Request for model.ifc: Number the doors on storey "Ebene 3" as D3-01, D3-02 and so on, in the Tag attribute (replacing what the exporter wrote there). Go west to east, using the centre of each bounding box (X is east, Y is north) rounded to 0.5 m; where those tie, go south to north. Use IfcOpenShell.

First a look at what the model holds.

```python
import ifcopenshell
import ifcopenshell.util.element
import ifcopenshell.util.placement

model = ifcopenshell.open("model.ifc")
print(model.schema)
storey = next(s for s in model.by_type("IfcBuildingStorey") if s.Name == "Ebene 3")
doors = [e for e in ifcopenshell.util.element.get_decomposition(storey) if e.is_a("IfcDoor")]
for e in sorted(doors, key=lambda e: e.id()):
    origin = ifcopenshell.util.placement.get_local_placement(e.ObjectPlacement)[:3, 3]
    print(e.id(), e.Tag, e.Name, origin.round(2) + 0.0, sep=" | ")
```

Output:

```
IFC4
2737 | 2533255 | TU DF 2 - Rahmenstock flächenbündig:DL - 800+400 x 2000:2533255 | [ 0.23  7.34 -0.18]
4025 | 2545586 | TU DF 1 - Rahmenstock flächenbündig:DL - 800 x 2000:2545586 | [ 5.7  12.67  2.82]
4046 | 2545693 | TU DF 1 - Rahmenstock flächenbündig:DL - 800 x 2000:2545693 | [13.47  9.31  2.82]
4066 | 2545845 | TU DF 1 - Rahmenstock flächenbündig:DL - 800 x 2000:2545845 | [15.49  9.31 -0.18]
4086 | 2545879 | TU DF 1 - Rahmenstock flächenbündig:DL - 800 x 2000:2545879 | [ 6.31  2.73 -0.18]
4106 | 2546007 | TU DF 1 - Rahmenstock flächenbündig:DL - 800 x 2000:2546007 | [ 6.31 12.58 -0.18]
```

```python
import ifcopenshell
import ifcopenshell.geom
import ifcopenshell.util.element
import ifcopenshell.util.shape

model = ifcopenshell.open("model.ifc")
settings = ifcopenshell.geom.settings()
settings.set("use-world-coords", True)


def centre(element):
    shape = ifcopenshell.geom.create_shape(settings, element)
    return ifcopenshell.util.shape.get_bbox_centroid(shape.geometry)


storey = next(s for s in model.by_type("IfcBuildingStorey") if s.Name == "Ebene 3")
doors = [e for e in ifcopenshell.util.element.get_decomposition(storey) if e.is_a("IfcDoor")]

# Insertion points can sit at a corner or the storey origin, so sort by the geometry (in metres).
centres = {e: centre(e) for e in doors}
doors.sort(key=lambda e: (round(centres[e][0] / 0.5), centres[e][1]))

for i, e in enumerate(doors, start=1):
    number = f"D3-{i:02d}"
    e.Tag = number
    print(e.id(), number)

model.write("model_v2.ifc")
```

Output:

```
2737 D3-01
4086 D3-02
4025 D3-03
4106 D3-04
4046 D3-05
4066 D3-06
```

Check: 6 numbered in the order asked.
